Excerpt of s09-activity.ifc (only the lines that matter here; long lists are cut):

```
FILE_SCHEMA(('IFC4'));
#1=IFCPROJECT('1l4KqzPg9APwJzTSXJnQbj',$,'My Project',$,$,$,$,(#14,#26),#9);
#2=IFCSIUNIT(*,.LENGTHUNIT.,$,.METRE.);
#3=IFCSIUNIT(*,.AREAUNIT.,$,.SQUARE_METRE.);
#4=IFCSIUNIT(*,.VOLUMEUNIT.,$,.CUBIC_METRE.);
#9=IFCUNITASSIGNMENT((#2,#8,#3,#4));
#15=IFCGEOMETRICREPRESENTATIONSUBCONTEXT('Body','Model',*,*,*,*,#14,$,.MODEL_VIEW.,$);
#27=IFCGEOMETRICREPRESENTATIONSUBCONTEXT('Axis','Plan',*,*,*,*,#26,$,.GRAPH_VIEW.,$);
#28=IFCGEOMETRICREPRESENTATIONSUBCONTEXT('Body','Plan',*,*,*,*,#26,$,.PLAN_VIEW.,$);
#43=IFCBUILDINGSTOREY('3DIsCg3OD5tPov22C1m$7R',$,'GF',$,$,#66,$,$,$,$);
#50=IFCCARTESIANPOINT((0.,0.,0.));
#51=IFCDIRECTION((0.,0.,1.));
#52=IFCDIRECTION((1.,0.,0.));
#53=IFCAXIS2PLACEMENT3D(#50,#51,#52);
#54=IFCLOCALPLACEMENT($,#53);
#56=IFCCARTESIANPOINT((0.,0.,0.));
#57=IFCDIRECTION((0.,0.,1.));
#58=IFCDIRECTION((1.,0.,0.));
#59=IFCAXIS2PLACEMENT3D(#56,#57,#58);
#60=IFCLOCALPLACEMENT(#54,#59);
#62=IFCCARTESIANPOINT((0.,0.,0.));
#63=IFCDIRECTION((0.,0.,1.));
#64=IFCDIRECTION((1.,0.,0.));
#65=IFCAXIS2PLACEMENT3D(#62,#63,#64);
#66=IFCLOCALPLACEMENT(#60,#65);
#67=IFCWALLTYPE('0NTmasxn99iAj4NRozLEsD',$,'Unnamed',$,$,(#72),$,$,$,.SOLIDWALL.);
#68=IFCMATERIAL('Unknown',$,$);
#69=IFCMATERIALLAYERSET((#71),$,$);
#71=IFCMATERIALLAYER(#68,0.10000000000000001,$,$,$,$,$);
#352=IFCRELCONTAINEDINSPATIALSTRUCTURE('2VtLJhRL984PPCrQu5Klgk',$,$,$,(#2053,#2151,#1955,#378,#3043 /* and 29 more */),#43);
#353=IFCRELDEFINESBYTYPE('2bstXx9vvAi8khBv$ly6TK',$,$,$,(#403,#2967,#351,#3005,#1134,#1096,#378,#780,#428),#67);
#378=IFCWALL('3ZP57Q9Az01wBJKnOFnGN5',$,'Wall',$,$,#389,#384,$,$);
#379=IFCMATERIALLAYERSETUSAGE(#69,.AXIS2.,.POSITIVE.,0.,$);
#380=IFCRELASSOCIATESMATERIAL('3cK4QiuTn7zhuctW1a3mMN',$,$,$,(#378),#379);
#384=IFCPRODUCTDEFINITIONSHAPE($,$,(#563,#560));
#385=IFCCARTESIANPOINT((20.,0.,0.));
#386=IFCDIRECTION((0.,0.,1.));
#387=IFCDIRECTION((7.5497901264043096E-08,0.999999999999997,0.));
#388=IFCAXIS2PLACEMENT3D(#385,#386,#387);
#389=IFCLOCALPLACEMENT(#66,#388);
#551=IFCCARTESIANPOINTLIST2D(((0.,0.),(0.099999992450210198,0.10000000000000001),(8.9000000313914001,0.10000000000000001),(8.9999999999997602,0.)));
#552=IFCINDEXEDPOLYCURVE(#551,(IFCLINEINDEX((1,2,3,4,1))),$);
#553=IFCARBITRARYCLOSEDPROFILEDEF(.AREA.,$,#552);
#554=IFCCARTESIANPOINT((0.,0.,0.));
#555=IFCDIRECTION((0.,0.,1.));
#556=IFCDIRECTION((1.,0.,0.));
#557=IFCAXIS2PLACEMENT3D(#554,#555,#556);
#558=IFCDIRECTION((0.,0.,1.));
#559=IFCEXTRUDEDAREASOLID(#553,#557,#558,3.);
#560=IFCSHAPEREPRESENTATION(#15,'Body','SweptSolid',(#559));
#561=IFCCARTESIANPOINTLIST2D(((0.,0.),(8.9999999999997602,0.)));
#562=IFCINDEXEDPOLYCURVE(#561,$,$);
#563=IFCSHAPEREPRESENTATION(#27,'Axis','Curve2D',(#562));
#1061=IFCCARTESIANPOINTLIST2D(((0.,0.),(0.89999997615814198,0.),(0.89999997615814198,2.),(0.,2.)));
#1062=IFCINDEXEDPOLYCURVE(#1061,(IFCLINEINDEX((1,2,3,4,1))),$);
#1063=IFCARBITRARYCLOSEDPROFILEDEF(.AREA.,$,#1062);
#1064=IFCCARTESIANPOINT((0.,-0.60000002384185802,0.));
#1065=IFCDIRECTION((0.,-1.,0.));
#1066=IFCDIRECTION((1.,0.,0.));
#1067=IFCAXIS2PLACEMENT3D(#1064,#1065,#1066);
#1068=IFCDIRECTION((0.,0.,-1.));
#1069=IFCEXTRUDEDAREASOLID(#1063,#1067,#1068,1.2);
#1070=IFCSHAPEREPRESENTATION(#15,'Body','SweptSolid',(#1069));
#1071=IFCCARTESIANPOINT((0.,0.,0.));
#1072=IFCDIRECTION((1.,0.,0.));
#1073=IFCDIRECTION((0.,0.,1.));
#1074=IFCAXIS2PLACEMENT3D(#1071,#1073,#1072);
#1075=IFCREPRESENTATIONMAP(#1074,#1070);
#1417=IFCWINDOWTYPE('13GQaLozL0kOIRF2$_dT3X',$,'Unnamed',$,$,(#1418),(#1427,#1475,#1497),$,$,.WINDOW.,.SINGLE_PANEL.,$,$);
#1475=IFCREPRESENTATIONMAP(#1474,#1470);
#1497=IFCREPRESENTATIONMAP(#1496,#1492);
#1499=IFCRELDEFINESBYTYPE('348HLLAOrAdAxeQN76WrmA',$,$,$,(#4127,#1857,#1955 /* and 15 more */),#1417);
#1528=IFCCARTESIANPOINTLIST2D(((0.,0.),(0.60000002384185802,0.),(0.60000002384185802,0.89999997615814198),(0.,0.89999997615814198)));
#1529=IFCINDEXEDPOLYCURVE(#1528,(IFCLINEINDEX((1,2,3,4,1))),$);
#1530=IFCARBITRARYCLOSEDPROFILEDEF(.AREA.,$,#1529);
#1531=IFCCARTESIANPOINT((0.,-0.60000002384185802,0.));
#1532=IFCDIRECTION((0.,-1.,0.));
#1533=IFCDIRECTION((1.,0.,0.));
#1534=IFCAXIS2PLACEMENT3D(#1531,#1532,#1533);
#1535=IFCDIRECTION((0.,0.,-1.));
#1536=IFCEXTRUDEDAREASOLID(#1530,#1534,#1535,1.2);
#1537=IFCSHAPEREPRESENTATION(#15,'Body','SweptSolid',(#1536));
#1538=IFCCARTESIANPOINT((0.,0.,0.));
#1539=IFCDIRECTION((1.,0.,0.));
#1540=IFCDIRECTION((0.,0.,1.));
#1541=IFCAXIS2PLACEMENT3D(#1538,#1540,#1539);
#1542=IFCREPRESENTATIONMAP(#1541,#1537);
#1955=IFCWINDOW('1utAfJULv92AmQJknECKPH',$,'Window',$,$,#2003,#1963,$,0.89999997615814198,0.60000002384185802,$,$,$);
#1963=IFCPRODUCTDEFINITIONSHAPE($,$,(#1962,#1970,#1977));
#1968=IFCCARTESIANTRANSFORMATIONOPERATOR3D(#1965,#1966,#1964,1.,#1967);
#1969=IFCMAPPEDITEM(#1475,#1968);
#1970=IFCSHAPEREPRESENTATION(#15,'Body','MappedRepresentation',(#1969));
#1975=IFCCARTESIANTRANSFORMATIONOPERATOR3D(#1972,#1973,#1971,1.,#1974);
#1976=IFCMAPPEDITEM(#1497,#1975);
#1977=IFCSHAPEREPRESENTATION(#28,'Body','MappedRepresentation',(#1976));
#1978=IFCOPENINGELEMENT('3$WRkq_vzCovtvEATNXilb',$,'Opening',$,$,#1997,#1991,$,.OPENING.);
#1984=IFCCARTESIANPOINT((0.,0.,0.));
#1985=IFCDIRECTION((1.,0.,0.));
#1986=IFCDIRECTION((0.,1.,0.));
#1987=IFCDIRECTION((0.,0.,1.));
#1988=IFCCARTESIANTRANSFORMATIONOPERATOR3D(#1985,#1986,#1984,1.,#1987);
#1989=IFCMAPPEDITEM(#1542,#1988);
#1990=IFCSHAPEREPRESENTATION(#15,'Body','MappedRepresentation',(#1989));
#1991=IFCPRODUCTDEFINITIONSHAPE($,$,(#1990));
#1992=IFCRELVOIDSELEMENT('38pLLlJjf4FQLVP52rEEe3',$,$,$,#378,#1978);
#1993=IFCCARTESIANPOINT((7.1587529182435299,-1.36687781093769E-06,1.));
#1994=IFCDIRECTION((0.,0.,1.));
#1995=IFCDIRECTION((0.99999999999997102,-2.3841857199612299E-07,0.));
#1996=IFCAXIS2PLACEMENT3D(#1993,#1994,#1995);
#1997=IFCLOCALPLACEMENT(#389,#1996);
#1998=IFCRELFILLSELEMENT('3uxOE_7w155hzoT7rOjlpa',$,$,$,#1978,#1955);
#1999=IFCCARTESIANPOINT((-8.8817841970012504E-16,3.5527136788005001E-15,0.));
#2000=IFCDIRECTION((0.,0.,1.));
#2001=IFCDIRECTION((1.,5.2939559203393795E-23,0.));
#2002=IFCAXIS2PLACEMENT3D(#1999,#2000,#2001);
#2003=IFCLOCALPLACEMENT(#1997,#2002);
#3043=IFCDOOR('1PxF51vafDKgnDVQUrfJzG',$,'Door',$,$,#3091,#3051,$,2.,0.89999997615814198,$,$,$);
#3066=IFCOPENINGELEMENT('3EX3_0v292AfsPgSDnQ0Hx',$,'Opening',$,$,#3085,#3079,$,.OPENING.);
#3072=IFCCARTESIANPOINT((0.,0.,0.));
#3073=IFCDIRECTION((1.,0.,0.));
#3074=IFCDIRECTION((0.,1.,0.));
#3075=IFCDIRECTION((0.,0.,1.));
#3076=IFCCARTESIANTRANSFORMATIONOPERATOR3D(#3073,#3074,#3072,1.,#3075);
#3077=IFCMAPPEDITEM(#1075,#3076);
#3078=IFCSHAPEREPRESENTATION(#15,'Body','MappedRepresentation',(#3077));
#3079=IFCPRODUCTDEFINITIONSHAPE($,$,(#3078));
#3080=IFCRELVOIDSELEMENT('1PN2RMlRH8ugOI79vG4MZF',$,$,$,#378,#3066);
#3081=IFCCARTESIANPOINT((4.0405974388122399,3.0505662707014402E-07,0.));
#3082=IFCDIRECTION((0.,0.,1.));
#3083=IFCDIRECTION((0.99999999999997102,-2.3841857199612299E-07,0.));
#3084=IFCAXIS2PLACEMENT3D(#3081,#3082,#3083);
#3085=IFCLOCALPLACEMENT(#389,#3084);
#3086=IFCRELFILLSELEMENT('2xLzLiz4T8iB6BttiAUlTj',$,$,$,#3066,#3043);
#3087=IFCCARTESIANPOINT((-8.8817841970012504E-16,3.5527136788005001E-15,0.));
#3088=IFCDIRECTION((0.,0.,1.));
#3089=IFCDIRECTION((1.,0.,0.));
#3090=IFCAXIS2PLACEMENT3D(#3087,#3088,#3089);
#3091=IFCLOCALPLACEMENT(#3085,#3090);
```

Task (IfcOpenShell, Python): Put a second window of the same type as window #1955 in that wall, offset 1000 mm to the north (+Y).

```python
import ifcopenshell
import ifcopenshell.api.feature
import ifcopenshell.api.geometry
import ifcopenshell.api.root
import ifcopenshell.geom
import ifcopenshell.util.element
import ifcopenshell.util.placement
import ifcopenshell.util.shape
import ifcopenshell.util.unit

model = ifcopenshell.open("s09-activity.ifc")
unit_scale = ifcopenshell.util.unit.calculate_unit_scale(model)
settings = ifcopenshell.geom.settings()


def volume(element):
    """Net volume in cubic metres, openings subtracted."""
    shape = ifcopenshell.geom.create_shape(settings, element)
    return ifcopenshell.util.shape.get_volume(shape.geometry)


window = model.by_id(1955)
opening = window.FillsVoids[0].RelatingOpeningElement
wall = opening.VoidsElements[0].RelatingBuildingElement
before = volume(wall)
shift = ifcopenshell.util.placement.get_local_placement(wall.ObjectPlacement)[:3, 0] * 1 / unit_scale

# copy_class copies the void relationship, type, container and properties, but no geometry.
new_opening = ifcopenshell.api.root.copy_class(model, product=opening)
new_opening.Representation = ifcopenshell.util.element.copy_deep(
    model, opening.Representation, exclude=["IfcGeometricRepresentationContext", "IfcRepresentationMap"]
)
new_window = ifcopenshell.api.root.copy_class(model, product=window)
new_window.Representation = ifcopenshell.util.element.copy_deep(
    model, window.Representation, exclude=["IfcGeometricRepresentationContext", "IfcRepresentationMap"]
)
ifcopenshell.api.feature.add_filling(model, opening=new_opening, element=new_window)

for old, new in ((opening, new_opening), (window, new_window)):
    matrix = ifcopenshell.util.placement.get_local_placement(old.ObjectPlacement)
    matrix[:3, 3] += shift
    ifcopenshell.api.geometry.edit_object_placement(model, product=new, matrix=matrix, is_si=False)

after = volume(wall)

print(f"wall volume {before:.3f} -> {after:.3f} m3")

model.write("s09-activity_edited.ifc")
```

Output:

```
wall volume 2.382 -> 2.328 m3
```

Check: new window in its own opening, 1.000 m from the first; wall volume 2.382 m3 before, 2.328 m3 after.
